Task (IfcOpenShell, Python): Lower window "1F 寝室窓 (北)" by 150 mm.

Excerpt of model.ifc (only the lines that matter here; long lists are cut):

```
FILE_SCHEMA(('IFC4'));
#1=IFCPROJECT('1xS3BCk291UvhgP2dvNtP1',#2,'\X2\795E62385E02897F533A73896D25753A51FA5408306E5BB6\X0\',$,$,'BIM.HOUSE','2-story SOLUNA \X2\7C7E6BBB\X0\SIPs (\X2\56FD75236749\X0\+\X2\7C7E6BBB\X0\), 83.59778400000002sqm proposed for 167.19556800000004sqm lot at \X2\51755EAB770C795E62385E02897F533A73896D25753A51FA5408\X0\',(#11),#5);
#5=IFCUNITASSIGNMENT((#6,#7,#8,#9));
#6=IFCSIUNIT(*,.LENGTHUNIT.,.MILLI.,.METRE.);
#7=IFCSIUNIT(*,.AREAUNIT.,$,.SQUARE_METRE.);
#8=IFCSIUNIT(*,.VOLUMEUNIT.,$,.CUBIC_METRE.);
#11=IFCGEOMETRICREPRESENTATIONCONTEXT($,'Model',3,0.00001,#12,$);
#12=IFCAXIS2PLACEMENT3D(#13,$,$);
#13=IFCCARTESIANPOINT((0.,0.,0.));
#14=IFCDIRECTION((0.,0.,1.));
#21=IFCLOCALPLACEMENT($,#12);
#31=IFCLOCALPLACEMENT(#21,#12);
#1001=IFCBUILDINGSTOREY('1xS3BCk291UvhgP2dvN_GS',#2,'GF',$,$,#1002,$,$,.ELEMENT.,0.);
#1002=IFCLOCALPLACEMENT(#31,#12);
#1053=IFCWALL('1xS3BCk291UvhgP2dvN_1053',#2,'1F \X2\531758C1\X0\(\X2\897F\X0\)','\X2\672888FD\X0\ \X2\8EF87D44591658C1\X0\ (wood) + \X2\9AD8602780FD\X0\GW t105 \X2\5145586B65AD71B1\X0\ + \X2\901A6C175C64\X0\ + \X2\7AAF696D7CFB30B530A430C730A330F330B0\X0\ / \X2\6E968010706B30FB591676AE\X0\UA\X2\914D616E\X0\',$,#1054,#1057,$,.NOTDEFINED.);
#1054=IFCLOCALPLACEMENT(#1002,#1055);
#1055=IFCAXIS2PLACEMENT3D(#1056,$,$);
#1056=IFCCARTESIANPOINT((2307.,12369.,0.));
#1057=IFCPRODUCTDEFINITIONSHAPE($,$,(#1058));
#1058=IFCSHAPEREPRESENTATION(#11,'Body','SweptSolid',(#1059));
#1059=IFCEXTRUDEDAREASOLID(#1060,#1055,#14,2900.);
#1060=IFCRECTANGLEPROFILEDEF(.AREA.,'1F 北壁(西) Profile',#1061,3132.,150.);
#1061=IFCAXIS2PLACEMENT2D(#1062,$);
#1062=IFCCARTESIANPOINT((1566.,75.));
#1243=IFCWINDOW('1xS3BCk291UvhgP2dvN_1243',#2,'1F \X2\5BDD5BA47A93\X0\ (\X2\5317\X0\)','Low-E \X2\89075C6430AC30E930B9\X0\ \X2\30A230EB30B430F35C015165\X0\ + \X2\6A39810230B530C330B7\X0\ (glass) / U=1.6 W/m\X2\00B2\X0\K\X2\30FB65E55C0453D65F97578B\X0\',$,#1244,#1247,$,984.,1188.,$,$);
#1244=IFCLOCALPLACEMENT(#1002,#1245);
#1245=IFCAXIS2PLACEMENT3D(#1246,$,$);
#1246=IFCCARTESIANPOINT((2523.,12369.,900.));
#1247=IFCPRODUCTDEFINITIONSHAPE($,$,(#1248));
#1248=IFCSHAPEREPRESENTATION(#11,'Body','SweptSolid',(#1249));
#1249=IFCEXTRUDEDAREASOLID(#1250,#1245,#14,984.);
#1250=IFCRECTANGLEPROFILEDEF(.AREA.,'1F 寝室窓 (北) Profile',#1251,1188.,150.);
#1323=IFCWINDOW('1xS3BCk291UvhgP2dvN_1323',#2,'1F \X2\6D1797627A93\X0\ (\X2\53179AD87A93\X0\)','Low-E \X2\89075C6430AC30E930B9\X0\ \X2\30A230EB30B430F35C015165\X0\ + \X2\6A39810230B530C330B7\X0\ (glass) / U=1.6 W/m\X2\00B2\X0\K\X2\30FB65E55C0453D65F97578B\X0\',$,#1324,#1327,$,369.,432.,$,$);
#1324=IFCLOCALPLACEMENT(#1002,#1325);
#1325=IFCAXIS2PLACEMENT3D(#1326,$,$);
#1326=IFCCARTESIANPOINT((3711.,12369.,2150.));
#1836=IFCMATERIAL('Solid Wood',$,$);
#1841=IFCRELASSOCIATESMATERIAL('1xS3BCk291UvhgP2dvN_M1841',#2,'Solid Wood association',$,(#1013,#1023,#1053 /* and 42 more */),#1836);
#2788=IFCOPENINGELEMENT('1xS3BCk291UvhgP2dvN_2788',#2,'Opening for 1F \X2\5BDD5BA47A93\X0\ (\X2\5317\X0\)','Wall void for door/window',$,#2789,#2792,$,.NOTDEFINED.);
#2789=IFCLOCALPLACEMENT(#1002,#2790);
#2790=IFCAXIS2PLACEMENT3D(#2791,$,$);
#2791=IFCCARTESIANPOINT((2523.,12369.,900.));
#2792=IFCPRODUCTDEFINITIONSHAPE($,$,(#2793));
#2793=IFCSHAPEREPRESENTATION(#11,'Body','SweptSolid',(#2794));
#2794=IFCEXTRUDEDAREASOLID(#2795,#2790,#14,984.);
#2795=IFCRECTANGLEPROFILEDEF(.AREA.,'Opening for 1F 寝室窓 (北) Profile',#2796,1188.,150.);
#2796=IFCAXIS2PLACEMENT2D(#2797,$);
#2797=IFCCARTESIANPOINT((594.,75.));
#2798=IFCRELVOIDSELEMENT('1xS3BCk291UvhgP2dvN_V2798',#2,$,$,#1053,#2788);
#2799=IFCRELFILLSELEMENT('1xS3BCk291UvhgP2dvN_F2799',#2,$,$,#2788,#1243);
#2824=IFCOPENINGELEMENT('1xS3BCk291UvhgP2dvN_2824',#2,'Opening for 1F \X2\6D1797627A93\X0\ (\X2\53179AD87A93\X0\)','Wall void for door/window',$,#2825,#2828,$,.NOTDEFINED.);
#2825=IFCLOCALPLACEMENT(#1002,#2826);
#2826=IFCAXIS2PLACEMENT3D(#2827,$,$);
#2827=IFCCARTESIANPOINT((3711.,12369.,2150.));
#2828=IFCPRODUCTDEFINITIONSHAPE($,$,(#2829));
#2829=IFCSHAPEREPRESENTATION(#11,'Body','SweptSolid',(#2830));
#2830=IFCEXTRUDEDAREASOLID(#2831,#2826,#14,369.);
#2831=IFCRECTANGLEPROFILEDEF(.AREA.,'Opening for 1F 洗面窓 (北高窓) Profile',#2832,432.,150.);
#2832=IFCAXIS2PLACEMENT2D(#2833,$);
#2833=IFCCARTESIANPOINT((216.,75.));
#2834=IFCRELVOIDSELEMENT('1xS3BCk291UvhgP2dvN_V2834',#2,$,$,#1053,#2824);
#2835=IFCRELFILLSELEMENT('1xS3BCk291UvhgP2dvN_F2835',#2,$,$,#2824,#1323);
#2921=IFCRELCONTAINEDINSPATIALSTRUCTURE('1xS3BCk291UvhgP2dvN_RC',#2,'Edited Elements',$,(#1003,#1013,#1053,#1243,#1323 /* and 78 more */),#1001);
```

```python
import numpy as np
import ifcopenshell
import ifcopenshell.api.geometry
import ifcopenshell.util.placement
import ifcopenshell.util.unit

model = ifcopenshell.open("model.ifc")
unit_scale = ifcopenshell.util.unit.calculate_unit_scale(model)

window = model.by_id(1243)
opening = window.FillsVoids[0].RelatingOpeningElement
dz = -150.0

shift = np.array([0.0, 0.0, dz])
# The window is not placed relative to its opening, so move both.
for product in (opening, window):
    matrix = ifcopenshell.util.placement.get_local_placement(product.ObjectPlacement)
    matrix[:3, 3] += shift
    ifcopenshell.api.geometry.edit_object_placement(model, product=product, matrix=matrix, is_si=False)

print(f"moved by {dz * unit_scale:+.3f} m")

model.write("model_edited.ifc")
```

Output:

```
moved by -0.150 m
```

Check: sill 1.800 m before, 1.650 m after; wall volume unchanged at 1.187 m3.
